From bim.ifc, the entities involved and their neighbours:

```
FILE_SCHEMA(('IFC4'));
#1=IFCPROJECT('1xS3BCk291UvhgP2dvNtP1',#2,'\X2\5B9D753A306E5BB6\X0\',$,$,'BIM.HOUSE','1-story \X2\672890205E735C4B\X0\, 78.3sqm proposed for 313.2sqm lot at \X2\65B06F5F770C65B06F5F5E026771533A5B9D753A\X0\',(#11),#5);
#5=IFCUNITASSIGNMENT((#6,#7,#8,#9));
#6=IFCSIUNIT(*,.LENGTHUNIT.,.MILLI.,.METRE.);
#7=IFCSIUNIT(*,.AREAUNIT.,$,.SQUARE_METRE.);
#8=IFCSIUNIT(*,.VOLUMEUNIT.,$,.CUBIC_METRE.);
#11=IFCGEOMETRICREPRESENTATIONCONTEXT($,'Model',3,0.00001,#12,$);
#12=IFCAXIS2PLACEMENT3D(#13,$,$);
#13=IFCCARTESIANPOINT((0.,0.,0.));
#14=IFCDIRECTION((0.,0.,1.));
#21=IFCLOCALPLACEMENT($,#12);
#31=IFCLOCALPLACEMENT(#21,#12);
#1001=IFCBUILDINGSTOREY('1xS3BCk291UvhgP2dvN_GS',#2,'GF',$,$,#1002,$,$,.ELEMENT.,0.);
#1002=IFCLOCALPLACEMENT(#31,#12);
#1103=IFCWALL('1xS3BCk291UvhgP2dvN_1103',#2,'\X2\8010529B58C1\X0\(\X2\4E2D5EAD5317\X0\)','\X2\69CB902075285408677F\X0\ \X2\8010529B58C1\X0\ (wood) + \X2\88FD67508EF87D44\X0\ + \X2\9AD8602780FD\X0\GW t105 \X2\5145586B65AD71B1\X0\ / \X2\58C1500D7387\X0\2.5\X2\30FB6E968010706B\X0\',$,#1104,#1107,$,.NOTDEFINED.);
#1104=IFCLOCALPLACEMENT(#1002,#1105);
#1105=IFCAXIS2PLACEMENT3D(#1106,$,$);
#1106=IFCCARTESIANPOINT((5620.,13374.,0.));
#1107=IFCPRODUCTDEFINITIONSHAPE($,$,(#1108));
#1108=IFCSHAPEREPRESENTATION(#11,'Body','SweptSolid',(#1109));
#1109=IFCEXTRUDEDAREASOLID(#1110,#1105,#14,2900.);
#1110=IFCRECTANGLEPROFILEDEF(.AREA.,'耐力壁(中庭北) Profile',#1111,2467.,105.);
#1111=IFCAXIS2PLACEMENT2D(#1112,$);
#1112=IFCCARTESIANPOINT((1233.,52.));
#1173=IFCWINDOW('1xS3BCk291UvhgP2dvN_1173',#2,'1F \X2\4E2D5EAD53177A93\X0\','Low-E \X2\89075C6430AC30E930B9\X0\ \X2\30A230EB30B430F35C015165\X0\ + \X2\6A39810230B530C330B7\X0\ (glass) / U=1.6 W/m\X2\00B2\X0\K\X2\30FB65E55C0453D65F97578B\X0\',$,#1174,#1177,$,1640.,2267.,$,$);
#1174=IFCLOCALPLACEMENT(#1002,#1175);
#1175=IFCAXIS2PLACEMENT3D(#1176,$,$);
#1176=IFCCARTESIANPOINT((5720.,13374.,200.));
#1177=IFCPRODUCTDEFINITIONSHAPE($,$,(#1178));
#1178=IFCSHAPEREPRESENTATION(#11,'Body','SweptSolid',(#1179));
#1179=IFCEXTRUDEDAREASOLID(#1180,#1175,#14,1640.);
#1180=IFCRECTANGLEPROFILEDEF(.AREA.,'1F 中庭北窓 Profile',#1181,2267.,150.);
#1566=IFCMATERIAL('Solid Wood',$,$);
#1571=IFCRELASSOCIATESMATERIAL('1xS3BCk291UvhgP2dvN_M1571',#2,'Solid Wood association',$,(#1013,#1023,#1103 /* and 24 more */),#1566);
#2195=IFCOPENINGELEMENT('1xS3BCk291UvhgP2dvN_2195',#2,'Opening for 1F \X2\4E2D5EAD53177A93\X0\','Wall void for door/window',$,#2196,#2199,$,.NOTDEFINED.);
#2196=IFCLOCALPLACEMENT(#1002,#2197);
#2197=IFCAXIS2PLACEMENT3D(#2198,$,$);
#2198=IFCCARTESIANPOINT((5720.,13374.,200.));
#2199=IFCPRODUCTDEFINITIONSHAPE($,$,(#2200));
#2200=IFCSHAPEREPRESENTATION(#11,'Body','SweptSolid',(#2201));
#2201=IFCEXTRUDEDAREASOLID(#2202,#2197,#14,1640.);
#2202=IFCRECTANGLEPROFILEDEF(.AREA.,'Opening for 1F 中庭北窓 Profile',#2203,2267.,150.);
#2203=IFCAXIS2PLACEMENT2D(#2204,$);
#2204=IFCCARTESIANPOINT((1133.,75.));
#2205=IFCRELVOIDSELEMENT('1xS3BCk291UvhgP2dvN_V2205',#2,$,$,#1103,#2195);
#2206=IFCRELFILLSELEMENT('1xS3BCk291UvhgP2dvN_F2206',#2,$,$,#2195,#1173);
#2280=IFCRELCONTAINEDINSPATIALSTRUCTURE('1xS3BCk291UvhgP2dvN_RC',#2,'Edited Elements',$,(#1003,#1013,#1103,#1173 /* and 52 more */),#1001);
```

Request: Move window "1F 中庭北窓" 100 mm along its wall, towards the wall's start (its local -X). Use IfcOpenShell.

```python
import ifcopenshell
import ifcopenshell.api.geometry
import ifcopenshell.util.placement
import ifcopenshell.util.unit

model = ifcopenshell.open("bim.ifc")
unit_scale = ifcopenshell.util.unit.calculate_unit_scale(model)

window = model.by_id(1173)
opening = window.FillsVoids[0].RelatingOpeningElement
wall = opening.VoidsElements[0].RelatingBuildingElement

wall_matrix = ifcopenshell.util.placement.get_local_placement(wall.ObjectPlacement)
shift = wall_matrix[:3, 0] * -0.1 / unit_scale
before = ifcopenshell.util.placement.get_local_placement(window.ObjectPlacement)[:3, 3].copy()

# The window is not placed relative to its opening, so move both.
for product in (opening, window):
    matrix = ifcopenshell.util.placement.get_local_placement(product.ObjectPlacement)
    matrix[:3, 3] += shift
    ifcopenshell.api.geometry.edit_object_placement(model, product=product, matrix=matrix, is_si=False)

after = ifcopenshell.util.placement.get_local_placement(window.ObjectPlacement)[:3, 3]
print("window moved by", (after - before).round(3) + 0.0)

model.write("bim_updated.ifc")
```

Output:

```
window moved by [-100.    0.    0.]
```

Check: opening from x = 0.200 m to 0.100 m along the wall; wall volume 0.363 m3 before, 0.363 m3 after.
